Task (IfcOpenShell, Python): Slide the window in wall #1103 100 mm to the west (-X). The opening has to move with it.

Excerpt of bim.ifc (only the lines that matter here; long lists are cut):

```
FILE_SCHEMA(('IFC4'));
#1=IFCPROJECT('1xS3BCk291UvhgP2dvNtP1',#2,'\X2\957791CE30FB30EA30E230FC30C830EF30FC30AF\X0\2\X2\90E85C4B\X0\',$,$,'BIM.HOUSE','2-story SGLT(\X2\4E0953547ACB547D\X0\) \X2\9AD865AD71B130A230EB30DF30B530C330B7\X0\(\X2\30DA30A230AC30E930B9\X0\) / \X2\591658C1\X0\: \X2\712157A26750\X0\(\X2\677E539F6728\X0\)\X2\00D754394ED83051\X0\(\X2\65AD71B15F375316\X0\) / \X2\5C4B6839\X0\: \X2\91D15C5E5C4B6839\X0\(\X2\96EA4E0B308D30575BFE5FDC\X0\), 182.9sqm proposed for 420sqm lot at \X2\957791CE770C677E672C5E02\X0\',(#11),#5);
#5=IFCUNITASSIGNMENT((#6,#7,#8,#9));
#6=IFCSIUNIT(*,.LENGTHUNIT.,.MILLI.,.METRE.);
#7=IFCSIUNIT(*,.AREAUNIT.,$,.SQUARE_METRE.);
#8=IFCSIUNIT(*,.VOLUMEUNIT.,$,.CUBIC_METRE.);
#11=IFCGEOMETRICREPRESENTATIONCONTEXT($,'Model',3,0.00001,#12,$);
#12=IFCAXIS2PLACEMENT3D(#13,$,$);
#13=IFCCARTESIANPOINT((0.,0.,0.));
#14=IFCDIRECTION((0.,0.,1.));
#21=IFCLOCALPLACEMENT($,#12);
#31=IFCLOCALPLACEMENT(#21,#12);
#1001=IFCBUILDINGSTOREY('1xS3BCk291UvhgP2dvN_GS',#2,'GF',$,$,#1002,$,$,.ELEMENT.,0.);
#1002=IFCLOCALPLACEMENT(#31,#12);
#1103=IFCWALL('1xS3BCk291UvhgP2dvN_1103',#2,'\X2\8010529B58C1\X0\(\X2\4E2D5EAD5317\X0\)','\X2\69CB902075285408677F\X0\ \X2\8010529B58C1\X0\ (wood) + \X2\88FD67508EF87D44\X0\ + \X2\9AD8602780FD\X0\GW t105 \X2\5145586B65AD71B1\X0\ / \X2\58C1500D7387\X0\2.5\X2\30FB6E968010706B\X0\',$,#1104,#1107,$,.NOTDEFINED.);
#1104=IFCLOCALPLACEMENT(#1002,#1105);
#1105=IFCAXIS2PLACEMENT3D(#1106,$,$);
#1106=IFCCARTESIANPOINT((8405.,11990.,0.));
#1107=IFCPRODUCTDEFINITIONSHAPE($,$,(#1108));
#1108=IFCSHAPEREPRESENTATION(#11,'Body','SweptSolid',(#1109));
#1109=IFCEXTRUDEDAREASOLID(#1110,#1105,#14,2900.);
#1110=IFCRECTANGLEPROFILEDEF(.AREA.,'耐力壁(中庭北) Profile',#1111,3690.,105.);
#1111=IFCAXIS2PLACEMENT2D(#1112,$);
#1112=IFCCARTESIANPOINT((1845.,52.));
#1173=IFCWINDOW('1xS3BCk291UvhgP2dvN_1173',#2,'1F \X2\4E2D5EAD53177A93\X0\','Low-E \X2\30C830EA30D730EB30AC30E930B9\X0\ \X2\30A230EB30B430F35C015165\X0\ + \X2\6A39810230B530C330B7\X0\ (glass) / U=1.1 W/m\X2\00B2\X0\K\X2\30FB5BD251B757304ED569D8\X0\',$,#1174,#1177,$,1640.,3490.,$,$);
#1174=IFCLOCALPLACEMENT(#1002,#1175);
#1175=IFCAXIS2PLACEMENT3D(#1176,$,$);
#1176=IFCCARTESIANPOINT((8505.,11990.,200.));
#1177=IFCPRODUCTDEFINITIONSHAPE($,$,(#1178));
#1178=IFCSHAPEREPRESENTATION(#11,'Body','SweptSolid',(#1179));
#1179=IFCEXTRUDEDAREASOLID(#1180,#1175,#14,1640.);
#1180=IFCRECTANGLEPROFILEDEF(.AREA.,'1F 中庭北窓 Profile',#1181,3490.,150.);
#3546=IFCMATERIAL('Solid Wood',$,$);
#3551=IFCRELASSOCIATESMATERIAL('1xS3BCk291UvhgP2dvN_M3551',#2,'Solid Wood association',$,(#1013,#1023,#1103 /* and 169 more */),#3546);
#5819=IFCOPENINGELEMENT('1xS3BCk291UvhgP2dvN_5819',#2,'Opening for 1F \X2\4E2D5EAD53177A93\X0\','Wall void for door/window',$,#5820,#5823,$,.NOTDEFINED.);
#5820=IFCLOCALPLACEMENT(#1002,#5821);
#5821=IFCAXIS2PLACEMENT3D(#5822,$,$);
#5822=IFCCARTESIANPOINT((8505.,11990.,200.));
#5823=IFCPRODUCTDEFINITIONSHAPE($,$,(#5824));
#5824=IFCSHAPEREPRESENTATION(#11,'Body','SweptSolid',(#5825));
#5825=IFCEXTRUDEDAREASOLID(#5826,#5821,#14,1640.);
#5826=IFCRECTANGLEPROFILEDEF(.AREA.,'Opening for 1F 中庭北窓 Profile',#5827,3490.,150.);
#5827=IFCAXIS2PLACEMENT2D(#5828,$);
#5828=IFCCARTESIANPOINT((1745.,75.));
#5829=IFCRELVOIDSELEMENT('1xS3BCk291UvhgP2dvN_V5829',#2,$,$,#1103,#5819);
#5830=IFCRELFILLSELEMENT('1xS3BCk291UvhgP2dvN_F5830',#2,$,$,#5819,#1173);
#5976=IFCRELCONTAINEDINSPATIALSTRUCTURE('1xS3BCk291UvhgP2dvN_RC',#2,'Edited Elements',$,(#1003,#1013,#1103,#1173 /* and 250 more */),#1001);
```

```python
import ifcopenshell
import ifcopenshell.api.geometry
import ifcopenshell.util.placement

model = ifcopenshell.open("bim.ifc")

window = model.by_guid("1xS3BCk291UvhgP2dvN_1173")
opening = window.FillsVoids[0].RelatingOpeningElement
wall = opening.VoidsElements[0].RelatingBuildingElement

wall_matrix = ifcopenshell.util.placement.get_local_placement(wall.ObjectPlacement)
shift = wall_matrix[:3, 0] * -100.0
before = ifcopenshell.util.placement.get_local_placement(window.ObjectPlacement)[:3, 3].copy()

# The window is not placed relative to its opening, so move both.
for product in (opening, window):
    matrix = ifcopenshell.util.placement.get_local_placement(product.ObjectPlacement)
    matrix[:3, 3] += shift
    ifcopenshell.api.geometry.edit_object_placement(model, product=product, matrix=matrix, is_si=False)

after = ifcopenshell.util.placement.get_local_placement(window.ObjectPlacement)[:3, 3]
print("window moved by", (after - before).round(3) + 0.0)

model.write("bim-out.ifc")
```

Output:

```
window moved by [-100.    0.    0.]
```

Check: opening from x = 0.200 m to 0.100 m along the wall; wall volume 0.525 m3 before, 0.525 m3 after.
